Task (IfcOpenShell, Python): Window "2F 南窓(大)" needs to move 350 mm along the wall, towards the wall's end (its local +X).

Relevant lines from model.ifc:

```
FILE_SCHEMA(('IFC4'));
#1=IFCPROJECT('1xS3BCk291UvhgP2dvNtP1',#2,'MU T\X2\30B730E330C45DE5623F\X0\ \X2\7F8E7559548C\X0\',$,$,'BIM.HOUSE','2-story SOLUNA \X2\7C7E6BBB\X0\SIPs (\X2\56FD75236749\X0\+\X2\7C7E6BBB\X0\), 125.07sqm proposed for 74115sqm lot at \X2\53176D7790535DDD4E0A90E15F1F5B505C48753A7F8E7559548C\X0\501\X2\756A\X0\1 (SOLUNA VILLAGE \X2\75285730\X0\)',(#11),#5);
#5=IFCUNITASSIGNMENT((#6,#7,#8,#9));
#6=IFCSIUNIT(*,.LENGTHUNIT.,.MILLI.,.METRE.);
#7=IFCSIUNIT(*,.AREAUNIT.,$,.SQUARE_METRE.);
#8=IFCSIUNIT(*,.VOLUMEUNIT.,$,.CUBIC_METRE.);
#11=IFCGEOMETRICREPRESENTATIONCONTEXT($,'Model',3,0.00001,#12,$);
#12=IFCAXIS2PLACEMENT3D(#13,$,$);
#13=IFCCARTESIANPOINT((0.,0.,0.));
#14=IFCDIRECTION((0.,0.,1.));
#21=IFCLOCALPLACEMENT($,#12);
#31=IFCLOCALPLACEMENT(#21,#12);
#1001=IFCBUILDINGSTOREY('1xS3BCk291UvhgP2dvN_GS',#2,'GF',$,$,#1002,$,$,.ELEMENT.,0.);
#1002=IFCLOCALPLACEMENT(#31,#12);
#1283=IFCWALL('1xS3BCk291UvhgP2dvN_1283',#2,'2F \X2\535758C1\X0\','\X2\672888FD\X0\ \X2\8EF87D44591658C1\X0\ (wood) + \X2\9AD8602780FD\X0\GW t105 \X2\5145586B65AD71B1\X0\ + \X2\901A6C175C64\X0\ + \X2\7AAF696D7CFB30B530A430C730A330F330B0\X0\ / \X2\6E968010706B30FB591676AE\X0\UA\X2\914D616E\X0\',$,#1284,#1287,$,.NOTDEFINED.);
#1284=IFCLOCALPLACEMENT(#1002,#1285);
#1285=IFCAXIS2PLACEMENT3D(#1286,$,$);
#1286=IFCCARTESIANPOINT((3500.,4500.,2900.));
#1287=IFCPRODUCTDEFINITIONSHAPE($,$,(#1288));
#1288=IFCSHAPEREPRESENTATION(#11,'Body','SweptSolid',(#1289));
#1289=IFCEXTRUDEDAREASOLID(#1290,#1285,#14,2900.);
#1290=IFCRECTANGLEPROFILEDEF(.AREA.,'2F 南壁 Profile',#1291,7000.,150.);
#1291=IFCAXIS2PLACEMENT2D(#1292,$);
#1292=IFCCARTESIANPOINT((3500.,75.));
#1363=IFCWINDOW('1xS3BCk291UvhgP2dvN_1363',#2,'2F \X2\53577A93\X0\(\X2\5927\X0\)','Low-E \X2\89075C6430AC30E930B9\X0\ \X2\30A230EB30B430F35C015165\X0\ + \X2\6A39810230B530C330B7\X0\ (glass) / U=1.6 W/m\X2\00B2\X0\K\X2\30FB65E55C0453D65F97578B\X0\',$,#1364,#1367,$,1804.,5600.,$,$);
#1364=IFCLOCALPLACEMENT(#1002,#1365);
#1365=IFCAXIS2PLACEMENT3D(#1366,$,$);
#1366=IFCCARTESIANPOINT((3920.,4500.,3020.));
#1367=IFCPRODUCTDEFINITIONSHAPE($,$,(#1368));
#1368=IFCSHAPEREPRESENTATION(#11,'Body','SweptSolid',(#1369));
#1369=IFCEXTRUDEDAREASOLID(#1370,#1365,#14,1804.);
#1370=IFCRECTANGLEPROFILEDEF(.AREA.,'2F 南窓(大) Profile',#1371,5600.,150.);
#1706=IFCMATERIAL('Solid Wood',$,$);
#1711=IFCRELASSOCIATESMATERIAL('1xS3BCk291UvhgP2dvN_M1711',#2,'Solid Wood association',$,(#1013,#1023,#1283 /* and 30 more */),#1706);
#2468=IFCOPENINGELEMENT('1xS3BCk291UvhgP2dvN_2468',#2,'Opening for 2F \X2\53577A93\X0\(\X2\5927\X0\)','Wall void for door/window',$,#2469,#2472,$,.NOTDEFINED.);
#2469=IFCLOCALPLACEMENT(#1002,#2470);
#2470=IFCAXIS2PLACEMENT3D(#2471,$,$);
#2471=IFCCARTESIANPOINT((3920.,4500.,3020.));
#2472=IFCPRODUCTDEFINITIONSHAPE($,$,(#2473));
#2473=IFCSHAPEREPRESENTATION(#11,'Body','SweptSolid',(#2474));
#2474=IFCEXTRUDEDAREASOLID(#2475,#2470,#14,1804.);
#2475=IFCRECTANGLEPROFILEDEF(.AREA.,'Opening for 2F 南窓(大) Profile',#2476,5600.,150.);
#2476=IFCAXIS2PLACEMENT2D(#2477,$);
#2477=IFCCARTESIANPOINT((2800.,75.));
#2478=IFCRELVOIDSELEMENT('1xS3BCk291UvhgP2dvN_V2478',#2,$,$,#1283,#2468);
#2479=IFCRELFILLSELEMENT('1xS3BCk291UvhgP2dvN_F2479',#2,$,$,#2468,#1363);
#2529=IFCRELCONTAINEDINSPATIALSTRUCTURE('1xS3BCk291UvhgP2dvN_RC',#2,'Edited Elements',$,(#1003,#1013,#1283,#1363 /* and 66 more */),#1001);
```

```python
import ifcopenshell
import ifcopenshell.api.geometry
import ifcopenshell.util.placement
import ifcopenshell.util.unit

model = ifcopenshell.open("model.ifc")
unit_scale = ifcopenshell.util.unit.calculate_unit_scale(model)

window = model.by_guid("1xS3BCk291UvhgP2dvN_1363")
opening = window.FillsVoids[0].RelatingOpeningElement
wall = opening.VoidsElements[0].RelatingBuildingElement

wall_matrix = ifcopenshell.util.placement.get_local_placement(wall.ObjectPlacement)
shift = wall_matrix[:3, 0] * 0.35 / unit_scale
before = ifcopenshell.util.placement.get_local_placement(window.ObjectPlacement)[:3, 3].copy()

# The window is not placed relative to its opening, so move both.
for product in (opening, window):
    matrix = ifcopenshell.util.placement.get_local_placement(product.ObjectPlacement)
    matrix[:3, 3] += shift
    ifcopenshell.api.geometry.edit_object_placement(model, product=product, matrix=matrix, is_si=False)

after = ifcopenshell.util.placement.get_local_placement(window.ObjectPlacement)[:3, 3]
print("window moved by", (after - before).round(3) + 0.0)

model.write("model_updated.ifc")
```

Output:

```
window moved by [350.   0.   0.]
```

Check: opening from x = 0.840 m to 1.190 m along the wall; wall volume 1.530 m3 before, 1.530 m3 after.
